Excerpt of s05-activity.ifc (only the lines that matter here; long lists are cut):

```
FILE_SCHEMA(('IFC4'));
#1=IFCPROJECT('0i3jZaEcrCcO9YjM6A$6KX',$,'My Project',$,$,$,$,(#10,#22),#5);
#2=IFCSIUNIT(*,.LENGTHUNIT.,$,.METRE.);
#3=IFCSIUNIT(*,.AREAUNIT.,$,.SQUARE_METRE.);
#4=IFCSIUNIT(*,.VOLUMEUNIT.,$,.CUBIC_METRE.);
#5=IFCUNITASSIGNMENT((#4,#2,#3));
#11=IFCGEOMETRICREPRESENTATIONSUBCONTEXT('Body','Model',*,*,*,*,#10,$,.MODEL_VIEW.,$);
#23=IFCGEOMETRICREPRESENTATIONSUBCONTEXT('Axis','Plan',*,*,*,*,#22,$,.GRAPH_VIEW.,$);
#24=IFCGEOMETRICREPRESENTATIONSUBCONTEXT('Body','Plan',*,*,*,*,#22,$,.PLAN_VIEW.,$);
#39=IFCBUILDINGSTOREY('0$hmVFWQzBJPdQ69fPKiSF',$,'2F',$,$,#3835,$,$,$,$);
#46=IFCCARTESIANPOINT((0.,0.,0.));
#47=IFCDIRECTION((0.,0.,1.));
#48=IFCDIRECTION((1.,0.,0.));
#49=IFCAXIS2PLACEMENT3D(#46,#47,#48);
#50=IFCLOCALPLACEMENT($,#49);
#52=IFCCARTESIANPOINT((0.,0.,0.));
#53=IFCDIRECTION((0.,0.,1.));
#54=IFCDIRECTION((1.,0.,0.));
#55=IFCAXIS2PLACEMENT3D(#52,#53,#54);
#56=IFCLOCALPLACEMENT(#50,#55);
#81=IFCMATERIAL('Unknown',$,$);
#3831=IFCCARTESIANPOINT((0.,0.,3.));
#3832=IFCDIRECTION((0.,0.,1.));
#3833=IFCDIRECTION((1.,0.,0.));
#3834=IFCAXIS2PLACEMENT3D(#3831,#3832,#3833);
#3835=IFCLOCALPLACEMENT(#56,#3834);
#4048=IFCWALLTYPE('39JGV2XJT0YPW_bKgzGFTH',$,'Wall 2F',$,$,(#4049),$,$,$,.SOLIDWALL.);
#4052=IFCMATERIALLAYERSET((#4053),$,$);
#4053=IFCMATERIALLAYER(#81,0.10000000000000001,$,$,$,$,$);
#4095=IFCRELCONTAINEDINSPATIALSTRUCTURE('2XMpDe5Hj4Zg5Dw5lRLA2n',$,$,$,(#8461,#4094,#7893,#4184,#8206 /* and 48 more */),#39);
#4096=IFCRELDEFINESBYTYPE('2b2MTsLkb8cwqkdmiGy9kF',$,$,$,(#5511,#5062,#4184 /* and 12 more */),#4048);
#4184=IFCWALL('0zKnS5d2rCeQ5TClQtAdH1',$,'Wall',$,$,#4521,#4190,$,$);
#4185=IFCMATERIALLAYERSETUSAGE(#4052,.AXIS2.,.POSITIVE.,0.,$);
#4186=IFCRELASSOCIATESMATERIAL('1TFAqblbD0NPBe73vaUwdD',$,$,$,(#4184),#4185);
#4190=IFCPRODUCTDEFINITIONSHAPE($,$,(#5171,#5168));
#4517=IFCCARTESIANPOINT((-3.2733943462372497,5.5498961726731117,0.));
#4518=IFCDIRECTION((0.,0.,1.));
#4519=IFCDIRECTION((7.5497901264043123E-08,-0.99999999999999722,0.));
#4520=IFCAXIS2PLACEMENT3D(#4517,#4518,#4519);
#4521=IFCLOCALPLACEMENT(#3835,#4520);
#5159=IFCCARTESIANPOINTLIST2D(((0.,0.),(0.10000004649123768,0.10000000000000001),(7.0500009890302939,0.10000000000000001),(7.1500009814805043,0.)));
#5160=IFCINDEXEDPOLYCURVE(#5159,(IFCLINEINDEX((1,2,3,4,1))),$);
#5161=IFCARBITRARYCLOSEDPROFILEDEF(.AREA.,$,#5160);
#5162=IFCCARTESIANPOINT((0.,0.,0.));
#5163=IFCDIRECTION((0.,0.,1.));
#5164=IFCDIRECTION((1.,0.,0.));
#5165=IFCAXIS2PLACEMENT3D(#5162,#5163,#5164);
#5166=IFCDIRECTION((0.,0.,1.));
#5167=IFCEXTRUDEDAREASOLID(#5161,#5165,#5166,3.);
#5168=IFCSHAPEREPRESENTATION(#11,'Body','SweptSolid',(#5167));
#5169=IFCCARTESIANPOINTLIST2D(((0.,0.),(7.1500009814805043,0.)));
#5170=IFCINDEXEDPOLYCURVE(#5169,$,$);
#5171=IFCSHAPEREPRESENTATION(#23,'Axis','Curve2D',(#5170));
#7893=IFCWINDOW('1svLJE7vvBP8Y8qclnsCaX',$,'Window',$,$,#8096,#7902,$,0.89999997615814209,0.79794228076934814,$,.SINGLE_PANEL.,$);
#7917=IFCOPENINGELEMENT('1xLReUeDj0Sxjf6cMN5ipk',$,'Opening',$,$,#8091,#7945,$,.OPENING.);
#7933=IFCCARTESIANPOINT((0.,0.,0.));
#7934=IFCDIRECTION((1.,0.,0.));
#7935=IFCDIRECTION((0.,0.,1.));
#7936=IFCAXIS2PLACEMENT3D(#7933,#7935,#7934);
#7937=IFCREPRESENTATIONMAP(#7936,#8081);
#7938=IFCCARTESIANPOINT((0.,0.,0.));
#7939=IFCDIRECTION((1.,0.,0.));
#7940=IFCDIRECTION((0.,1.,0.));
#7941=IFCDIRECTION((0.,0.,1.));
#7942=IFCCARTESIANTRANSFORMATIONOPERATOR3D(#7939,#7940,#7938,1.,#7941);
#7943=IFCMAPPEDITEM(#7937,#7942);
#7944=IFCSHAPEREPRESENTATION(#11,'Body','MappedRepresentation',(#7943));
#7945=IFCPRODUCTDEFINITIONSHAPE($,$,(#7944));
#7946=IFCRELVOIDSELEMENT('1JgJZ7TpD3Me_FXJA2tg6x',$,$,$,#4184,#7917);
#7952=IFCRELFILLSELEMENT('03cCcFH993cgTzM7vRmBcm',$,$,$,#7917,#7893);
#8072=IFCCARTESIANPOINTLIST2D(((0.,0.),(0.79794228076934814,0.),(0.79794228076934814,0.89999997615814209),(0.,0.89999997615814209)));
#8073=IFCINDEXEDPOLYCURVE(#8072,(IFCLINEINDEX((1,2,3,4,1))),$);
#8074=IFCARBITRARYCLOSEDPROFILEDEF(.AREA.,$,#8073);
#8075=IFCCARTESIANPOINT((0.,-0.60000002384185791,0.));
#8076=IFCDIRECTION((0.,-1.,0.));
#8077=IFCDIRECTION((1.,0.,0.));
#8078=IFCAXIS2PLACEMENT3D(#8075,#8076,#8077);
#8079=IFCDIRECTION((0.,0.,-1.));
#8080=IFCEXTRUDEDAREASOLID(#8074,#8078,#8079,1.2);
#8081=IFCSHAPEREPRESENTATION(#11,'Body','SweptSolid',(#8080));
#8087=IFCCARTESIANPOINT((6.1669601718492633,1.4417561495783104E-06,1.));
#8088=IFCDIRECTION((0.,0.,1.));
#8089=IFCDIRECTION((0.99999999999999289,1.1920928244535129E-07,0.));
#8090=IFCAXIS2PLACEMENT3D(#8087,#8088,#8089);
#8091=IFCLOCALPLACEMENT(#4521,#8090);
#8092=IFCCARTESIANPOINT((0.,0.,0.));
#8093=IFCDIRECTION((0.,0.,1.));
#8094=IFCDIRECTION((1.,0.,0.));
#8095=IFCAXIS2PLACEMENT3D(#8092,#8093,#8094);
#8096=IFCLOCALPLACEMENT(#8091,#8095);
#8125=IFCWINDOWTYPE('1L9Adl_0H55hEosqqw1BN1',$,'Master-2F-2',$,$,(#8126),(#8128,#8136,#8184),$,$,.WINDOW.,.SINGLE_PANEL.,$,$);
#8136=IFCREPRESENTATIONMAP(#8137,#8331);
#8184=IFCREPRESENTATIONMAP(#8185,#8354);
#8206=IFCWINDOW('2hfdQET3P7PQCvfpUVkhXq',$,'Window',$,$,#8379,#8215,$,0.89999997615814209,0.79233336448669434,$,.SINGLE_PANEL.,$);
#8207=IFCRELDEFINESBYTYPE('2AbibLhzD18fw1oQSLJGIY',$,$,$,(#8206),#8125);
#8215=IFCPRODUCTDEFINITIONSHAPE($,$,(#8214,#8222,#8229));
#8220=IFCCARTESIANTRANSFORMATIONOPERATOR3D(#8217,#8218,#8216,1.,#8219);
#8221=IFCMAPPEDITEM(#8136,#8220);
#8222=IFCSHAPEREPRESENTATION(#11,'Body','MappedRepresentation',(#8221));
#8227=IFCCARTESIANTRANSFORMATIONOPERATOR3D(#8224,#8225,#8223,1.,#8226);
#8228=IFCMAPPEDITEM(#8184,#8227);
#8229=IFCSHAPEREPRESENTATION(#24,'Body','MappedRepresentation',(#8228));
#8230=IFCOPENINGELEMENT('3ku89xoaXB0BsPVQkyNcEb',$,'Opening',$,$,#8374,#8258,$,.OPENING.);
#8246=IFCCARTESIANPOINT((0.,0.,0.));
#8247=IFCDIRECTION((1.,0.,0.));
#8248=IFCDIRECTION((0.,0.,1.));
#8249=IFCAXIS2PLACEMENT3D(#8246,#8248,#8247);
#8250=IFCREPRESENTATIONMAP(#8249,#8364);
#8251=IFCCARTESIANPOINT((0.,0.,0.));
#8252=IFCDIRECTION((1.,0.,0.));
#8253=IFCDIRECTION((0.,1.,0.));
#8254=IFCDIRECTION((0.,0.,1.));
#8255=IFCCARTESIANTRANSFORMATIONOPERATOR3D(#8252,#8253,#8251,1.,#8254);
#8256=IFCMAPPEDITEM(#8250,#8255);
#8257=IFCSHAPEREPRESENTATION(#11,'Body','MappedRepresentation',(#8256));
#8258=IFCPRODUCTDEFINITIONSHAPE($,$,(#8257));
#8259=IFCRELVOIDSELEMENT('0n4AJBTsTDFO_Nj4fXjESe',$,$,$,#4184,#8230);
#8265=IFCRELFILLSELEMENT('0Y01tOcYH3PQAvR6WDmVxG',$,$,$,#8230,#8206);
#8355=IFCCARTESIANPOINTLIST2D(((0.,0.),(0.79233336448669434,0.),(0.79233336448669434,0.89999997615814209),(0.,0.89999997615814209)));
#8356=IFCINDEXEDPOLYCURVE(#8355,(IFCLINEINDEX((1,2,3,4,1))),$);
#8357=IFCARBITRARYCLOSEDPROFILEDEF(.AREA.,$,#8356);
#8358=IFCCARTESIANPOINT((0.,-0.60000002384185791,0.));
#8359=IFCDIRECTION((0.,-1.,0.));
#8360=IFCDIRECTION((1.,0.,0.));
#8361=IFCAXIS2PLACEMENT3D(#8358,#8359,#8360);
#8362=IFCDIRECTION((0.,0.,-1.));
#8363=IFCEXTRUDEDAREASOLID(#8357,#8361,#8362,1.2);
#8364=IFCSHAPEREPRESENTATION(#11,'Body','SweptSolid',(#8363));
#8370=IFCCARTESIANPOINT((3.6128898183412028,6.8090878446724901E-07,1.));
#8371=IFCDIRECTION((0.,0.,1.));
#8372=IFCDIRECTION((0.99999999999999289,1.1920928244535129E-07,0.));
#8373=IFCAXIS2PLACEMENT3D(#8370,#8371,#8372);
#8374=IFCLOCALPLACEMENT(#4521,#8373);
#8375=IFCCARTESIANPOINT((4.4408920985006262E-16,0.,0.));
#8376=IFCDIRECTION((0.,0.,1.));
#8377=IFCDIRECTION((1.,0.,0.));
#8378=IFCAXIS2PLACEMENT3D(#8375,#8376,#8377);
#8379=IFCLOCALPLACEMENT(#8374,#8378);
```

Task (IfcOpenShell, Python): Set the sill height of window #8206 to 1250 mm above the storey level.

```python
import numpy as np
import ifcopenshell
import ifcopenshell.api.geometry
import ifcopenshell.geom
import ifcopenshell.util.element
import ifcopenshell.util.placement
import ifcopenshell.util.shape
import ifcopenshell.util.unit

model = ifcopenshell.open("s05-activity.ifc")
unit_scale = ifcopenshell.util.unit.calculate_unit_scale(model)

window = model.by_id(8206)
opening = window.FillsVoids[0].RelatingOpeningElement
storey = ifcopenshell.util.element.get_container(window, ifc_class="IfcBuildingStorey")
level = ifcopenshell.util.placement.get_local_placement(storey.ObjectPlacement)[2, 3]

# The opening's origin need not be at the sill, so measure its lowest point.
shape = ifcopenshell.geom.create_shape(ifcopenshell.geom.settings(), opening)
bottom = ifcopenshell.util.shape.get_shape_bottom_elevation(shape, shape.geometry) / unit_scale
dz = level + 1.25 / unit_scale - bottom

shift = np.array([0.0, 0.0, dz])
# The window is placed relative to its opening, so it follows when the opening moves.
matrix = ifcopenshell.util.placement.get_local_placement(opening.ObjectPlacement)
matrix[:3, 3] += shift
ifcopenshell.api.geometry.edit_object_placement(
    model, product=opening, matrix=matrix, is_si=False, should_transform_children=True
)

print(f"moved by {dz * unit_scale:+.3f} m")

model.write("s05-activity_updated.ifc")
```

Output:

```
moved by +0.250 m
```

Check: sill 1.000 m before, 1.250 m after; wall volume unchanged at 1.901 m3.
